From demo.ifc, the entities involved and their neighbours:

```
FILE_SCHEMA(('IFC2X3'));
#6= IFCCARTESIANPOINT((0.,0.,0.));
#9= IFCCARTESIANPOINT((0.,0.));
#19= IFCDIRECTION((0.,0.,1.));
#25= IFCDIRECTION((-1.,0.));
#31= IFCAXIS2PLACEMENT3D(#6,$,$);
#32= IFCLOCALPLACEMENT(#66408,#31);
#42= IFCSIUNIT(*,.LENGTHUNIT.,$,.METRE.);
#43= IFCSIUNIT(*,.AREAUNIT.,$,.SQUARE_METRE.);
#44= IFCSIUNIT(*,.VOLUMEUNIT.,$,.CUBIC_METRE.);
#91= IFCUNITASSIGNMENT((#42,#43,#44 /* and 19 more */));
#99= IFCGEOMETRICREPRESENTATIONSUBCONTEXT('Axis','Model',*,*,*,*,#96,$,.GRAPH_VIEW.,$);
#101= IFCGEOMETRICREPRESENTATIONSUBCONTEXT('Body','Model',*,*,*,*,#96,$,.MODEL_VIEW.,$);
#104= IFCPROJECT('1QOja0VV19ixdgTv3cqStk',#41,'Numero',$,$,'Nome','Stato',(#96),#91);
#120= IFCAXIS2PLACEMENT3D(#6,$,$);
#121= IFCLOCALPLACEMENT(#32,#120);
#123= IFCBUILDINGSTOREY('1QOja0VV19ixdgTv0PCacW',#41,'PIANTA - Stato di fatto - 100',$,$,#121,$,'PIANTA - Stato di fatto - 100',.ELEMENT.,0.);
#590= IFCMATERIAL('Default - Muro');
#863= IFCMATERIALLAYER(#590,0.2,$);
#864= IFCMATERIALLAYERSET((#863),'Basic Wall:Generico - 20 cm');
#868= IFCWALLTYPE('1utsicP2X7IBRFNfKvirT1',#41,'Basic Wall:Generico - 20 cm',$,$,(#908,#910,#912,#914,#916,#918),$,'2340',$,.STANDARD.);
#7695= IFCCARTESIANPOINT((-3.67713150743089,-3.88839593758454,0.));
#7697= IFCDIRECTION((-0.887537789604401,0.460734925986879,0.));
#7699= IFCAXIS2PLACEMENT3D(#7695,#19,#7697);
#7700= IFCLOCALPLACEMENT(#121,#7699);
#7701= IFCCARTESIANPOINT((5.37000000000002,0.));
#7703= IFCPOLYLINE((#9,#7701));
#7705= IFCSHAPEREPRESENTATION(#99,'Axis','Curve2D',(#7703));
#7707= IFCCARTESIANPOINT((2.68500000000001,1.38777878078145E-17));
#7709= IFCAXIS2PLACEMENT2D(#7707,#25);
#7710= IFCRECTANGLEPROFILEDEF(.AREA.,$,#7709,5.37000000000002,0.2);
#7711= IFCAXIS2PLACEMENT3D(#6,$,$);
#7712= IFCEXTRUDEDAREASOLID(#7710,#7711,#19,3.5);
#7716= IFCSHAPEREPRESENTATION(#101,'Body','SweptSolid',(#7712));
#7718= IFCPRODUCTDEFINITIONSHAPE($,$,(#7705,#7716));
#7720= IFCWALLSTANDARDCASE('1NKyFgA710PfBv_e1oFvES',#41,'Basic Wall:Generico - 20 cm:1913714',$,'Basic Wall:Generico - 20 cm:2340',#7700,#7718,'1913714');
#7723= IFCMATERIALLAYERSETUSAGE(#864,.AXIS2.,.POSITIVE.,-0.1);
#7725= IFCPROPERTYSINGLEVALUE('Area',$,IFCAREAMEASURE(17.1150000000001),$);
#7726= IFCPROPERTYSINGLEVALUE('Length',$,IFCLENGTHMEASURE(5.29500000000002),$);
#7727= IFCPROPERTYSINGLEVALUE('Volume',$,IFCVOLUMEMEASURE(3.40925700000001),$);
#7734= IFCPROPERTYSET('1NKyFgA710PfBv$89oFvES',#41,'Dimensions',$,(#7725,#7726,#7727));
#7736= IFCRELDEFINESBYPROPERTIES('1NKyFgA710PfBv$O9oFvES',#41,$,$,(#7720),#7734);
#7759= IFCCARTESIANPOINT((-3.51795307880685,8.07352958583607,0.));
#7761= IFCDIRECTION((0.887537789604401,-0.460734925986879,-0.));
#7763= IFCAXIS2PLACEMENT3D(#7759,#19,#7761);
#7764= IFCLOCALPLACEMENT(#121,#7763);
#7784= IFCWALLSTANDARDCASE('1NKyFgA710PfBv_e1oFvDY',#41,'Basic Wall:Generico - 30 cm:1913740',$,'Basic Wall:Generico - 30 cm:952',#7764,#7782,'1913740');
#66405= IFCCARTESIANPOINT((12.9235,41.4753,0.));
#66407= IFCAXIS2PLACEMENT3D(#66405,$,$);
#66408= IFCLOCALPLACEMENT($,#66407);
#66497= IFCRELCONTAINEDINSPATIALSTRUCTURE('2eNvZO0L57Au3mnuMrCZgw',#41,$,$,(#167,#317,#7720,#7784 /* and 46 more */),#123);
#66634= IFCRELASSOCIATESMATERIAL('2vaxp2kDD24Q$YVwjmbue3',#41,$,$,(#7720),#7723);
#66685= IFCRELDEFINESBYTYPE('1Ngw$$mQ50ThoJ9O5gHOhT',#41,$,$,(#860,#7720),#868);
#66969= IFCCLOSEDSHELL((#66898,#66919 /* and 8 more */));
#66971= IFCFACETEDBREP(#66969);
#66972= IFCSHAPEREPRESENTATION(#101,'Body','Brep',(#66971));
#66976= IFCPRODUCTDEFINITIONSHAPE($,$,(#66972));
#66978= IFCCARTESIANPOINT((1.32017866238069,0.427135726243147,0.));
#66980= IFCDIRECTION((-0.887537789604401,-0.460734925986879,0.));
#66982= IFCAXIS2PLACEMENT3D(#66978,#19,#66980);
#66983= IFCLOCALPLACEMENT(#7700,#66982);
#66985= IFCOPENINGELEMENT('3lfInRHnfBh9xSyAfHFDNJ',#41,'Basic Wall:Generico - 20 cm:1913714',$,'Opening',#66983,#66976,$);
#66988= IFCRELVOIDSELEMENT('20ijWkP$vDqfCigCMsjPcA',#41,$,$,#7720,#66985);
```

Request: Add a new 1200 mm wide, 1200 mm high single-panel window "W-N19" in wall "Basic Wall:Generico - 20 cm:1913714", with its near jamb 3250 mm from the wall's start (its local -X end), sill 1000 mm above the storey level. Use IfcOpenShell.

```python
import numpy as np
import ifcopenshell
import ifcopenshell.api.feature
import ifcopenshell.api.geometry
import ifcopenshell.api.pset
import ifcopenshell.api.root
import ifcopenshell.api.spatial
import ifcopenshell.api.type
import ifcopenshell.geom
import ifcopenshell.util.element
import ifcopenshell.util.placement
import ifcopenshell.util.representation
import ifcopenshell.util.shape
import ifcopenshell.util.unit

model = ifcopenshell.open("demo.ifc")
unit_scale = ifcopenshell.util.unit.calculate_unit_scale(model)
area_scale = ifcopenshell.util.unit.calculate_unit_scale(model, "AREAUNIT")
volume_scale = ifcopenshell.util.unit.calculate_unit_scale(model, "VOLUMEUNIT")
settings = ifcopenshell.geom.settings()


def volume(element):
    """Net volume in cubic metres, openings subtracted."""
    shape = ifcopenshell.geom.create_shape(settings, element)
    return ifcopenshell.util.shape.get_volume(shape.geometry)


wall = model.by_guid("1NKyFgA710PfBv_e1oFvES")
storey = ifcopenshell.util.element.get_container(wall, ifc_class="IfcBuildingStorey")
context = ifcopenshell.util.representation.get_context(model, "Model", "Body", "MODEL_VIEW")
before = volume(wall)

width, height, from_end, sill = 1.2, 1.2, 3.25, 1  # metres

# The wall runs along its own X axis, and the end named is its -X end.
wall_shape = ifcopenshell.geom.create_shape(settings, wall)
x, y, z = ifcopenshell.util.shape.get_vertices(wall_shape.geometry).T
start = x.min() + from_end
face, thickness = float(y.min()), float(y.max() - y.min())
wall_matrix = ifcopenshell.util.placement.get_local_placement(wall.ObjectPlacement)
level = ifcopenshell.util.placement.get_local_placement(storey.ObjectPlacement)[2, 3]


def in_wall(x, y):
    """Placement at x, y metres in the wall's axes, at sill height."""
    matrix = wall_matrix.copy()
    matrix[:, 3] = wall_matrix @ np.array([x / unit_scale, y / unit_scale, 0.0, 1.0])
    matrix[2, 3] = level + sill / unit_scale
    return matrix


# Opening: a box that overshoots both wall faces by 50 mm.
opening = ifcopenshell.api.root.create_entity(model, ifc_class="IfcOpeningElement")
box = ifcopenshell.api.geometry.add_wall_representation(
    model, context=context, length=width, height=height, thickness=thickness + 0.1
)
ifcopenshell.api.geometry.assign_representation(model, product=opening, representation=box)
ifcopenshell.api.geometry.edit_object_placement(model, product=opening, matrix=in_wall(start, face - 0.05), is_si=False)
ifcopenshell.api.feature.add_feature(model, feature=opening, element=wall)

window = ifcopenshell.api.root.create_entity(model, ifc_class="IfcWindow", name="W-N19")
window.OverallWidth, window.OverallHeight = width / unit_scale, height / unit_scale
body = ifcopenshell.api.geometry.add_window_representation(
    model,
    context=context,
    overall_width=window.OverallWidth,
    overall_height=window.OverallHeight,
    partition_type="SINGLE_PANEL",
)
ifcopenshell.api.geometry.assign_representation(model, product=window, representation=body)
ifcopenshell.api.spatial.assign_container(model, products=[window], relating_structure=storey)
fills = ifcopenshell.api.feature.add_filling(model, opening=opening, element=window)
fills.OwnerHistory = window.OwnerHistory  # required in IFC2X3

# IFC2X3 keeps the operation on the window style.
style = ifcopenshell.api.root.create_entity(model, ifc_class="IfcWindowStyle", name="W-N19")
style.OperationType, style.ConstructionType = "SINGLE_PANEL", "NOTDEFINED"
style.ParameterTakesPrecedence = style.Sizeable = False
ifcopenshell.api.type.assign_type(model, related_objects=[window], relating_type=style)

# Centre the window in the wall's thickness.
ifcopenshell.api.geometry.edit_object_placement(model, product=window, matrix=in_wall(start, face), is_si=False)
window_shape = ifcopenshell.geom.create_shape(settings, window)
depth = ifcopenshell.util.shape.get_vertices(window_shape.geometry)[:, 1]
offset = face + thickness / 2 - (depth.min() + depth.max()) / 2
ifcopenshell.api.geometry.edit_object_placement(model, product=window, matrix=in_wall(start, offset), is_si=False)

after = volume(wall)

# Update the wall's stored quantities.
pset = model.by_id(ifcopenshell.util.element.get_pset(wall, "Dimensions", should_inherit=False)["id"])
ifcopenshell.api.pset.edit_pset(model, pset=pset, properties={
    "Area": model.create_entity("IfcAreaMeasure", after / thickness / area_scale),
    "Volume": model.create_entity("IfcVolumeMeasure", after / volume_scale),
})

print(f"wall volume {before:.3f} -> {after:.3f} m3")

model.write("demo_edited.ifc")
```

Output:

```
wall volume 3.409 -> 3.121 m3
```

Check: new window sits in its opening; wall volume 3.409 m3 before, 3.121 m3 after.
